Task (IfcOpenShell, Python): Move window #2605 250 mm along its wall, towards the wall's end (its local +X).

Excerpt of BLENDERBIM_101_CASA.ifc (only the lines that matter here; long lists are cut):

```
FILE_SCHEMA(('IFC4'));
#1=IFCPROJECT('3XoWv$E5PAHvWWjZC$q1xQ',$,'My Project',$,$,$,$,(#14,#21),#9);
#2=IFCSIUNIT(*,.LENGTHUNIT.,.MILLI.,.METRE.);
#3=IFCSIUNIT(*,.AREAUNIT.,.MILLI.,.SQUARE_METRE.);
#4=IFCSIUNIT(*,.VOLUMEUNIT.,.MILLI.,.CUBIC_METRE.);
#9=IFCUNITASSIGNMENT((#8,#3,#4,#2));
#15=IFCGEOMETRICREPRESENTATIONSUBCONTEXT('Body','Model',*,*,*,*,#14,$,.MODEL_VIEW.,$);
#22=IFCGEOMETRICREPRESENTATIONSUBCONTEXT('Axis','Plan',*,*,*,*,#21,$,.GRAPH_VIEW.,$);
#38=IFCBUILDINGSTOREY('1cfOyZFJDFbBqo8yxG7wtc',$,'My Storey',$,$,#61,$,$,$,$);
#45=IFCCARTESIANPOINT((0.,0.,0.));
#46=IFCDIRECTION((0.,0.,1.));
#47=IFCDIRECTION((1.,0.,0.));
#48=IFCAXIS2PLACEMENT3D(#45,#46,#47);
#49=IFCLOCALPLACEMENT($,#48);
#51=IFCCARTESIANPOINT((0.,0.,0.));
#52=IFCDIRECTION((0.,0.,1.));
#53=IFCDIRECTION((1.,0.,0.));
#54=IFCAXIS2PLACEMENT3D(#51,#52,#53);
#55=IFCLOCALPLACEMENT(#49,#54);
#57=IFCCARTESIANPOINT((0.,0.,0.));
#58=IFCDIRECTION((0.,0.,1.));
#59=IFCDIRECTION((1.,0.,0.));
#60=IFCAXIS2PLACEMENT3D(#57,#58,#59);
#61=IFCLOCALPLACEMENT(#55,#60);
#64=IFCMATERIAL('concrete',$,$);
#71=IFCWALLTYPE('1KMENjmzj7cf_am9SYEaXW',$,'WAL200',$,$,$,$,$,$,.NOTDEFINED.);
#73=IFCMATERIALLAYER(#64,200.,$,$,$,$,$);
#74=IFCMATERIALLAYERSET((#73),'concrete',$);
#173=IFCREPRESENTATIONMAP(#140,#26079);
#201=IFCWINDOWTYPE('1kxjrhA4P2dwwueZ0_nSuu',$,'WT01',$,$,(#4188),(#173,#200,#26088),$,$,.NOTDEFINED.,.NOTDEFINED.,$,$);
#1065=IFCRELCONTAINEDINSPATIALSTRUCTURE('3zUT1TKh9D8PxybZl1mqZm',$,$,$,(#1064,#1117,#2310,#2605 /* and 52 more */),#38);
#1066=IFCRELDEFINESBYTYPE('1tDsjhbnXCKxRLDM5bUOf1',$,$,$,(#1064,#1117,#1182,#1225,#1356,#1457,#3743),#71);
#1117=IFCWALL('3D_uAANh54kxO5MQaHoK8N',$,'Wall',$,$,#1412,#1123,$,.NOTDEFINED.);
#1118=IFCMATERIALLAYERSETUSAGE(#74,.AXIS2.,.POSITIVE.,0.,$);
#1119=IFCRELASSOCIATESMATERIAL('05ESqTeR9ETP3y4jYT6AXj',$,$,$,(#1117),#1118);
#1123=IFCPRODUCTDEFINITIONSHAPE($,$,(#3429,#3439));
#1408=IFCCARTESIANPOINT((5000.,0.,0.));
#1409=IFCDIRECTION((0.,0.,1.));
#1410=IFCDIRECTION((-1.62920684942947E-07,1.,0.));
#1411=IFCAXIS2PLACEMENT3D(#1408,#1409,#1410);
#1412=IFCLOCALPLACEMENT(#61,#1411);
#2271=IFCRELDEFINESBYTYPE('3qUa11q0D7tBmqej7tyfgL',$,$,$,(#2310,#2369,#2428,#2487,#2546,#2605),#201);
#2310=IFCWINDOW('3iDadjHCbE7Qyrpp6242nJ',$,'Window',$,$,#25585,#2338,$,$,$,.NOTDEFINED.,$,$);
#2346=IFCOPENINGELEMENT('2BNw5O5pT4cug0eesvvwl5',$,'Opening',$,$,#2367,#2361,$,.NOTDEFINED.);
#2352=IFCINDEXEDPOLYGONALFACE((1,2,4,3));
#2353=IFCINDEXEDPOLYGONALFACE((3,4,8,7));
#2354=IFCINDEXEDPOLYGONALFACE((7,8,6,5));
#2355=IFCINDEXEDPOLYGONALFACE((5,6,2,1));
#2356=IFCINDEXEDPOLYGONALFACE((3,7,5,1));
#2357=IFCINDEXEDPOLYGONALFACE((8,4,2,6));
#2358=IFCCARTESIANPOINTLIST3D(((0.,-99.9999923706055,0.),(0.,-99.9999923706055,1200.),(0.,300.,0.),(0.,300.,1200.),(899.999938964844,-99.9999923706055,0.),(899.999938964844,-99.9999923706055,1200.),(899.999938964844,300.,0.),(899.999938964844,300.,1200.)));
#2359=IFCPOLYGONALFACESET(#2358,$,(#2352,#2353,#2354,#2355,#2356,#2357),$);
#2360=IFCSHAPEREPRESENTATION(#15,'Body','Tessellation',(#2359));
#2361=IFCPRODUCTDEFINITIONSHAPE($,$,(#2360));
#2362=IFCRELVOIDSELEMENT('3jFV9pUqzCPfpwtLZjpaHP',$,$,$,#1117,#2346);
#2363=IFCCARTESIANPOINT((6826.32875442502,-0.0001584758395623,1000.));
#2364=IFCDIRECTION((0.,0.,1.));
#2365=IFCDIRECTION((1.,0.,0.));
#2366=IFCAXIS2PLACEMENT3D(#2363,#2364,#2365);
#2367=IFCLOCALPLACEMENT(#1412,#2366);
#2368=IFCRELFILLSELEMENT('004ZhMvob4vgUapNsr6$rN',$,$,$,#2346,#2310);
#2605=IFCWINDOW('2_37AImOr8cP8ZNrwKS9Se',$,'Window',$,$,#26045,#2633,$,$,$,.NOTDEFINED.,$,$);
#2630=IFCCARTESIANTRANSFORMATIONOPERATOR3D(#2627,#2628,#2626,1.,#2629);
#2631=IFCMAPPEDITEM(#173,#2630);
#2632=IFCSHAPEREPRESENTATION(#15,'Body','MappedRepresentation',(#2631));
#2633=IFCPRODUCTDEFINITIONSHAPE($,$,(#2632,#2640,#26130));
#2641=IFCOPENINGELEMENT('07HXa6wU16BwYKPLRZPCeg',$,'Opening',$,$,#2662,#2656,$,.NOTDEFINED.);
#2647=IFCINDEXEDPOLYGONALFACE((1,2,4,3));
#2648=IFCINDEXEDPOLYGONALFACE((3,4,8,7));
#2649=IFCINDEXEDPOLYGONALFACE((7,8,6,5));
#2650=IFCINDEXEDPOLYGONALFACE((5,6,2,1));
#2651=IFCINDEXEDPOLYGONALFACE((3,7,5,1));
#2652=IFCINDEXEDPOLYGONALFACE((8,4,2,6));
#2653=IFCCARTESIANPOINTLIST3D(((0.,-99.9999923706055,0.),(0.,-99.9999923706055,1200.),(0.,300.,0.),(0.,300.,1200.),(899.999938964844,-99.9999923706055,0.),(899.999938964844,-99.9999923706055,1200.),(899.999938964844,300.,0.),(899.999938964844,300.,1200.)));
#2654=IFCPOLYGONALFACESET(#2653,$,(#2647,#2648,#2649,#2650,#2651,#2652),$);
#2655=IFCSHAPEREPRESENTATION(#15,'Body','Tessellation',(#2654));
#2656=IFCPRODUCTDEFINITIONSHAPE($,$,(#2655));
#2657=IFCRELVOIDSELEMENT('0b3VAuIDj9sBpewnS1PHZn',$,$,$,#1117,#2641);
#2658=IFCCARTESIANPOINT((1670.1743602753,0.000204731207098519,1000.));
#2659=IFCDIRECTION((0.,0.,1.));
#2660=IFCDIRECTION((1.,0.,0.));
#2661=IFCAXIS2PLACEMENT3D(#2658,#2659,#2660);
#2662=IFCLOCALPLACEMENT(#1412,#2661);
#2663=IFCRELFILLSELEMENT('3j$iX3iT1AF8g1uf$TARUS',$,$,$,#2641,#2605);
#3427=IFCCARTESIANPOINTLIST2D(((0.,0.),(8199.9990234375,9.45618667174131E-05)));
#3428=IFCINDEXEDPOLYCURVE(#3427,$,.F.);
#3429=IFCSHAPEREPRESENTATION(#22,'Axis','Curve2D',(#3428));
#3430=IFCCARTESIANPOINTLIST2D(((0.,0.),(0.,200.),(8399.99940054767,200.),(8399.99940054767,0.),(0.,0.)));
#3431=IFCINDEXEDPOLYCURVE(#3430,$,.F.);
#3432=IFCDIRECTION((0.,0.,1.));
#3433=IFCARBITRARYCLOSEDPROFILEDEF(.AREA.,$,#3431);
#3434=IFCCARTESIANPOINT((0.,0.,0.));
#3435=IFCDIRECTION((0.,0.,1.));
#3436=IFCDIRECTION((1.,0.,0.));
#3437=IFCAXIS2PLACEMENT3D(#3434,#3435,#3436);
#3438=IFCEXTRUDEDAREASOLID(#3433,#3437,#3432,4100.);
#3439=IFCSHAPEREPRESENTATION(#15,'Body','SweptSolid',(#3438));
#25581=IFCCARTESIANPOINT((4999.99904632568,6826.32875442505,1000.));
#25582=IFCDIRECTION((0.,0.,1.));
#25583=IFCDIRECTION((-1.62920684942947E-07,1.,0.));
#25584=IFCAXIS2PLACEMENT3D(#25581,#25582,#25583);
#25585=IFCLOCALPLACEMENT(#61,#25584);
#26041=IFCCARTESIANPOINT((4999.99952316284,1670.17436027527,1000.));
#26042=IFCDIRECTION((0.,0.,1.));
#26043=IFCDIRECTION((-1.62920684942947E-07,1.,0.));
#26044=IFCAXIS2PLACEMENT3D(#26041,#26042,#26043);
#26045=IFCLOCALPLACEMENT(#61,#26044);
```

```python
import ifcopenshell
import ifcopenshell.api.geometry
import ifcopenshell.util.placement
import ifcopenshell.util.unit

model = ifcopenshell.open("BLENDERBIM_101_CASA.ifc")
unit_scale = ifcopenshell.util.unit.calculate_unit_scale(model)

window = model.by_guid("2_37AImOr8cP8ZNrwKS9Se")
opening = window.FillsVoids[0].RelatingOpeningElement
wall = opening.VoidsElements[0].RelatingBuildingElement

wall_matrix = ifcopenshell.util.placement.get_local_placement(wall.ObjectPlacement)
shift = wall_matrix[:3, 0] * 0.25 / unit_scale
before = ifcopenshell.util.placement.get_local_placement(window.ObjectPlacement)[:3, 3].copy()

# The window is not placed relative to its opening, so move both.
for product in (opening, window):
    matrix = ifcopenshell.util.placement.get_local_placement(product.ObjectPlacement)
    matrix[:3, 3] += shift
    ifcopenshell.api.geometry.edit_object_placement(model, product=product, matrix=matrix, is_si=False)

after = ifcopenshell.util.placement.get_local_placement(window.ObjectPlacement)[:3, 3]
print("window moved by", (after - before).round(3) + 0.0)

model.write("BLENDERBIM_101_CASA_updated.ifc")
```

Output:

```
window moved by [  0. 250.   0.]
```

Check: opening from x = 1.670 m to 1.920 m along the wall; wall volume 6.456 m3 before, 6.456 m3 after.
